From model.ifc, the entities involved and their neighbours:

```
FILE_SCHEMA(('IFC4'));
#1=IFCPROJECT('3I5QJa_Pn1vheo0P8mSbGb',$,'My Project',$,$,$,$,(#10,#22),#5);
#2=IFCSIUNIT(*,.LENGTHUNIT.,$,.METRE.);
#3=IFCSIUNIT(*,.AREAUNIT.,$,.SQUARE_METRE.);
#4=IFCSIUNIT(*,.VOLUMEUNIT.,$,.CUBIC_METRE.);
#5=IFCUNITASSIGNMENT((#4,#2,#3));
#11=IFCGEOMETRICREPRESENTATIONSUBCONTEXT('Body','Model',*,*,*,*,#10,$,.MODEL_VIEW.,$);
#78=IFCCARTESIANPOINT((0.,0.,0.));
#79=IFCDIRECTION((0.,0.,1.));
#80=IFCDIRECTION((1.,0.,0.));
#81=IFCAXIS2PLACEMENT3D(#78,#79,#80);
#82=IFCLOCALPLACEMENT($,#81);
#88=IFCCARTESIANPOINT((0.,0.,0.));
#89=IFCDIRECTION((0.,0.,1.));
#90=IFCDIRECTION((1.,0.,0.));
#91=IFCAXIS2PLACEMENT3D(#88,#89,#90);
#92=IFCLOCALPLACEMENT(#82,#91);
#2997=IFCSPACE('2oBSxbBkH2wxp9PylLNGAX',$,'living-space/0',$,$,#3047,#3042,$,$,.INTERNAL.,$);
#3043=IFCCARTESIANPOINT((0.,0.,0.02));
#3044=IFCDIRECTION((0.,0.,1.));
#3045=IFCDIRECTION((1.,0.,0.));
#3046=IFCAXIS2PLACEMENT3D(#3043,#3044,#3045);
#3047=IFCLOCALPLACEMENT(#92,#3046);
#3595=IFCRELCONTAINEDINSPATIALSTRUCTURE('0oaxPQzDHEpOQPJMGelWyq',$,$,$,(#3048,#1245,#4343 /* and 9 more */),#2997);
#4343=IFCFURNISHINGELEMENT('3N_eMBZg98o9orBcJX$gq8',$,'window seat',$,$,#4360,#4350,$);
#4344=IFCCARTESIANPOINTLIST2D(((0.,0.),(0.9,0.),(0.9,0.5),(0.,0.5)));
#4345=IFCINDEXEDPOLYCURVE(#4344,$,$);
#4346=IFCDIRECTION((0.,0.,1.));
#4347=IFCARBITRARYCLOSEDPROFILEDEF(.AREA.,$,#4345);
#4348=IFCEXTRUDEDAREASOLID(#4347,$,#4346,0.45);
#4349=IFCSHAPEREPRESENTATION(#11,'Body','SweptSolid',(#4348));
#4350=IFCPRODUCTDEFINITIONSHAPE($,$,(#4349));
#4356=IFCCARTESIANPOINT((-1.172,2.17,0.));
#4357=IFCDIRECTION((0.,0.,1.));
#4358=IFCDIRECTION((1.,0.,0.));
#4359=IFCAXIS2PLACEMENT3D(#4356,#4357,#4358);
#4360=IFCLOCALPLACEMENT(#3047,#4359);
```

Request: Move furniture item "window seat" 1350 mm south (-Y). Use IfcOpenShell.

```python
import ifcopenshell
import ifcopenshell.api.geometry
import ifcopenshell.util.placement

model = ifcopenshell.open("model.ifc")

item = model.by_guid("3N_eMBZg98o9orBcJX$gq8")
matrix = ifcopenshell.util.placement.get_local_placement(item.ObjectPlacement)
matrix[1, 3] -= 1.35
ifcopenshell.api.geometry.edit_object_placement(model, product=item, matrix=matrix, is_si=False)

print(ifcopenshell.util.placement.get_local_placement(item.ObjectPlacement).round(3) + 0.0)

model.write("model_rev.ifc")
```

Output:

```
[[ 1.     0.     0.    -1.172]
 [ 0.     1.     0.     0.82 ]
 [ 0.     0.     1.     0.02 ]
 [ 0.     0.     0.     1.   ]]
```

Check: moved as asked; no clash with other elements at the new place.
